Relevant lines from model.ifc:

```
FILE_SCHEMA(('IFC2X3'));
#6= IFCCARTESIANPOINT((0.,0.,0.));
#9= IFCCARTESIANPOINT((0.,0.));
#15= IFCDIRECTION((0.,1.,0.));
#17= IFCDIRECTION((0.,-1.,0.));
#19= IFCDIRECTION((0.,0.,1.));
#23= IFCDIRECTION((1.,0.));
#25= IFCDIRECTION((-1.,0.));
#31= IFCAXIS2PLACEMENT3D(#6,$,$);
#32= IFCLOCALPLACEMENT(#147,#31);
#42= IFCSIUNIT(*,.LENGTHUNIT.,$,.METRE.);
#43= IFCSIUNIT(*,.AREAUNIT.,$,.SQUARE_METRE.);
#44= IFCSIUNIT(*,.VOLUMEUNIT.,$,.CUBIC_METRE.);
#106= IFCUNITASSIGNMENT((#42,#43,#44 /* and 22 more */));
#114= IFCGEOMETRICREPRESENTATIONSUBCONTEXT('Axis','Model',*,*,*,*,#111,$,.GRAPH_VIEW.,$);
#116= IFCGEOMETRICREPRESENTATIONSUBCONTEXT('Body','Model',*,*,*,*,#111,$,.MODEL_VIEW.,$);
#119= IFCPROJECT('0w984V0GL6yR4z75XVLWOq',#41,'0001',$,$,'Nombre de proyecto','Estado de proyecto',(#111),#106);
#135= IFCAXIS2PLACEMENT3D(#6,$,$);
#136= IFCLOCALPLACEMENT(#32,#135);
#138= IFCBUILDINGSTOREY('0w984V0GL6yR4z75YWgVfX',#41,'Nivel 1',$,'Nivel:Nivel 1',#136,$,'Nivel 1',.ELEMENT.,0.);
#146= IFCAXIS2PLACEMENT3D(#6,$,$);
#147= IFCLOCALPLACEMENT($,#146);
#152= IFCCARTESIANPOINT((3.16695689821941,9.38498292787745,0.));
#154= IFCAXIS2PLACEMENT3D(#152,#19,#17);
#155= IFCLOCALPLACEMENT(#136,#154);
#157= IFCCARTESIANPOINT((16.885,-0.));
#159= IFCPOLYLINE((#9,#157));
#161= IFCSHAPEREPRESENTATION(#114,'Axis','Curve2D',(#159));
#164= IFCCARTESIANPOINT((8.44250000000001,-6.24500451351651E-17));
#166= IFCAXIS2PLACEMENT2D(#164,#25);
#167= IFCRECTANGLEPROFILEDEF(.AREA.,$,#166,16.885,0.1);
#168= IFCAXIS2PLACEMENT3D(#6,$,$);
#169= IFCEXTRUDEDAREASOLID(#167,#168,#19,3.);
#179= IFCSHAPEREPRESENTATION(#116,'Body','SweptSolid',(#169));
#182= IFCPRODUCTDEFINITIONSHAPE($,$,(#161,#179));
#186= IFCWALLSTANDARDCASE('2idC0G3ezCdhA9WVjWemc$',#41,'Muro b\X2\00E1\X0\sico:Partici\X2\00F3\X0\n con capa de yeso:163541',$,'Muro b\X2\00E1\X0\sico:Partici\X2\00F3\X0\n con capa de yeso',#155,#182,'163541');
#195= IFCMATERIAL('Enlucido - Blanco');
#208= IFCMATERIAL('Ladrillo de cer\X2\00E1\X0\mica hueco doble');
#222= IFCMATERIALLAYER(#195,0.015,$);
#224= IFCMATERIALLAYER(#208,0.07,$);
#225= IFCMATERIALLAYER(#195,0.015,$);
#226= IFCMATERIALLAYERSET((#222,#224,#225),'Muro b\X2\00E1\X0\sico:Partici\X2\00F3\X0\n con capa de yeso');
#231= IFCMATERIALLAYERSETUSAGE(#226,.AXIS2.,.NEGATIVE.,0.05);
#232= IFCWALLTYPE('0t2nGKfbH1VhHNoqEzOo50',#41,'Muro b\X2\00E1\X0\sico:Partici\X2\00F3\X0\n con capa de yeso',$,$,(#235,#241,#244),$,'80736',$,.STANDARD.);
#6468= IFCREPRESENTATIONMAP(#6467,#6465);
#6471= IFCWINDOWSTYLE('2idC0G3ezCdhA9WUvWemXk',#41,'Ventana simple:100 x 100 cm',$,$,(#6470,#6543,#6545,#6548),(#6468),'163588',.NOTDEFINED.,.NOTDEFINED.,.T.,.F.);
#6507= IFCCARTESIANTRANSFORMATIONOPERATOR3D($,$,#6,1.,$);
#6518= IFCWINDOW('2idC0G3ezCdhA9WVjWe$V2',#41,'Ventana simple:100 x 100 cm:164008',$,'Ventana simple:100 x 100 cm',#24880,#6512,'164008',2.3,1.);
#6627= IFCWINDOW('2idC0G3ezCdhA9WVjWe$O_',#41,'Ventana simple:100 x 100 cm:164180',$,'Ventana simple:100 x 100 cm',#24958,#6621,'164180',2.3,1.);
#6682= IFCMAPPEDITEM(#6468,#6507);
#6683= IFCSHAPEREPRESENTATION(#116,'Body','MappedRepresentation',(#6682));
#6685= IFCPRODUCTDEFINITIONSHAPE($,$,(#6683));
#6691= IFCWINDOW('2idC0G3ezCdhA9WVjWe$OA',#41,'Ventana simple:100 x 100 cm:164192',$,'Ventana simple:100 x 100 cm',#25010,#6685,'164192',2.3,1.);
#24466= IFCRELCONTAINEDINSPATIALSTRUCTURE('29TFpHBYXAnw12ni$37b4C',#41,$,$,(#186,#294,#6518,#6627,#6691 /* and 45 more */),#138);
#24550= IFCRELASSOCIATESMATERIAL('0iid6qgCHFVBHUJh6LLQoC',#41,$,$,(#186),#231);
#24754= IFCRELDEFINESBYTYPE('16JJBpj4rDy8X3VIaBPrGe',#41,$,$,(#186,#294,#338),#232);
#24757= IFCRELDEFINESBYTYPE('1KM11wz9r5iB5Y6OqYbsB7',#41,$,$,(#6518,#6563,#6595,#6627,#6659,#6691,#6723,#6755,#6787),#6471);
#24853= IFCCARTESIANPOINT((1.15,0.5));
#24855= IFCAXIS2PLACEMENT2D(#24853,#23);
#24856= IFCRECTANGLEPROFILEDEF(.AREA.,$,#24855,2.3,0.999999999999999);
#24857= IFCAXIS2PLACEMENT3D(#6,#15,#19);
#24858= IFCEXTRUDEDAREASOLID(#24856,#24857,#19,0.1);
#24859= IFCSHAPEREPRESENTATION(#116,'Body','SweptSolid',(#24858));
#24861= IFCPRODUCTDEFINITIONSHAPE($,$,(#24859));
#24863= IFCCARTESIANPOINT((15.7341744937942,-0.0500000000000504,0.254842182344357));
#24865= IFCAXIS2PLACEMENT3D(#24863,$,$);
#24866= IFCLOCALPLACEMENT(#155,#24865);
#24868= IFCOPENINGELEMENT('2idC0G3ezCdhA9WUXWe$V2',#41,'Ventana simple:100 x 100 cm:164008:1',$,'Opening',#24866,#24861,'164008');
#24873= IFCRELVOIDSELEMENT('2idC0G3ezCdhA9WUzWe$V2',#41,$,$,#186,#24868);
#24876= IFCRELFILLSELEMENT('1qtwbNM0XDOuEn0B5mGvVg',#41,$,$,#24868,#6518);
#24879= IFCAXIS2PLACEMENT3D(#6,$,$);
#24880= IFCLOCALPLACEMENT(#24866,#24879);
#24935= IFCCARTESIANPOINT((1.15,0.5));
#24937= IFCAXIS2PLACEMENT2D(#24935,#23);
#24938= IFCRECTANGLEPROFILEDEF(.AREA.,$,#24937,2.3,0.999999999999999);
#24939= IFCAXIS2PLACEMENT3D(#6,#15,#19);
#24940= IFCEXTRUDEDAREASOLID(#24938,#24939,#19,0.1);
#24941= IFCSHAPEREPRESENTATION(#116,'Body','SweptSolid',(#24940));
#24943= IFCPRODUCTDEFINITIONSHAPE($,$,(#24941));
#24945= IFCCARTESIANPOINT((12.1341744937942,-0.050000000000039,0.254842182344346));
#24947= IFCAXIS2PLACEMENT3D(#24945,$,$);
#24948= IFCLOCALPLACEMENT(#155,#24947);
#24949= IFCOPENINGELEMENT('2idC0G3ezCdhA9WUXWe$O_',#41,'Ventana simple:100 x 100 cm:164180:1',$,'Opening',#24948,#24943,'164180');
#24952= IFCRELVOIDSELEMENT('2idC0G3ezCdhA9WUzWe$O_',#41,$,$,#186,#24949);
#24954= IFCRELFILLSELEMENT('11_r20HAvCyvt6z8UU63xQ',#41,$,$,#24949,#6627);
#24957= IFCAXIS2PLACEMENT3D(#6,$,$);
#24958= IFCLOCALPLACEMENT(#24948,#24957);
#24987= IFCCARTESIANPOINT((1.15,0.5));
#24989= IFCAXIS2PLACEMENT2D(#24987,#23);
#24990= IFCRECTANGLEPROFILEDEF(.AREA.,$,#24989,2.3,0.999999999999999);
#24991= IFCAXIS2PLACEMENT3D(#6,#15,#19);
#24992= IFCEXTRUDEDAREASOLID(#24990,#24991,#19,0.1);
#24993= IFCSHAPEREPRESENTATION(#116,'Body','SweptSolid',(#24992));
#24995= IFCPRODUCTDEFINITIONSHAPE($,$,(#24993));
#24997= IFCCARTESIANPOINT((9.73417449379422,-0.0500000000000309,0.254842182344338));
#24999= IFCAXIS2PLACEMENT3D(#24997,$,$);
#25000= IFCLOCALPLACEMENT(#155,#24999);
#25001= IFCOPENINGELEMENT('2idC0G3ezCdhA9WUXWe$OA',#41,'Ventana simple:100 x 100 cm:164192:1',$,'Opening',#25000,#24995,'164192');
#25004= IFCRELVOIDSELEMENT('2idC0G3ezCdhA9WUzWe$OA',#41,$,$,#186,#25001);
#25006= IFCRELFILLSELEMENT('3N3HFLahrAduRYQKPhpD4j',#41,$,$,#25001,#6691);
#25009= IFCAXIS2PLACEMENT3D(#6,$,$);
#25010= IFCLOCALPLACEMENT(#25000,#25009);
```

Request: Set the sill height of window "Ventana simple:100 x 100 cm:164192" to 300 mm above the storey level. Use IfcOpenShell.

```python
import numpy as np
import ifcopenshell
import ifcopenshell.api.geometry
import ifcopenshell.geom
import ifcopenshell.util.element
import ifcopenshell.util.placement
import ifcopenshell.util.shape
import ifcopenshell.util.unit

model = ifcopenshell.open("model.ifc")
unit_scale = ifcopenshell.util.unit.calculate_unit_scale(model)

window = model.by_guid("2idC0G3ezCdhA9WVjWe$OA")
opening = window.FillsVoids[0].RelatingOpeningElement
storey = ifcopenshell.util.element.get_container(window, ifc_class="IfcBuildingStorey")
level = ifcopenshell.util.placement.get_local_placement(storey.ObjectPlacement)[2, 3]

# The opening's origin need not be at the sill, so measure its lowest point.
shape = ifcopenshell.geom.create_shape(ifcopenshell.geom.settings(), opening)
bottom = ifcopenshell.util.shape.get_shape_bottom_elevation(shape, shape.geometry) / unit_scale
dz = level + 0.3 - bottom

shift = np.array([0.0, 0.0, dz])
# The window is placed relative to its opening, so it follows when the opening moves.
matrix = ifcopenshell.util.placement.get_local_placement(opening.ObjectPlacement)
matrix[:3, 3] += shift
ifcopenshell.api.geometry.edit_object_placement(
    model, product=opening, matrix=matrix, is_si=False, should_transform_children=True
)

print(f"moved by {dz * unit_scale:+.3f} m")

model.write("model_rev.ifc")
```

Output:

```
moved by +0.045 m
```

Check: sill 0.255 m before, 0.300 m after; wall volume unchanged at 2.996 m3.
